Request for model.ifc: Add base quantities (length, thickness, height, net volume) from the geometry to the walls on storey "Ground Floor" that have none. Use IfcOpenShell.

First a look at what the model holds.

```python
import ifcopenshell
import ifcopenshell.util.element
import ifcopenshell.util.unit

model = ifcopenshell.open("model.ifc")
print(model.schema)
for unit_type in ("LENGTHUNIT", "AREAUNIT", "VOLUMEUNIT"):
    print(unit_type, ifcopenshell.util.unit.calculate_unit_scale(model, unit_type))
storey = next(s for s in model.by_type("IfcBuildingStorey") if s.Name == "Ground Floor")
walls = [e for e in ifcopenshell.util.element.get_decomposition(storey) if e.is_a("IfcWall")]
for e in sorted(walls, key=lambda e: e.id()):
    print(e.id(), e.is_a(), e.Name, list(ifcopenshell.util.element.get_psets(e, qtos_only=True)), sep=" | ")
```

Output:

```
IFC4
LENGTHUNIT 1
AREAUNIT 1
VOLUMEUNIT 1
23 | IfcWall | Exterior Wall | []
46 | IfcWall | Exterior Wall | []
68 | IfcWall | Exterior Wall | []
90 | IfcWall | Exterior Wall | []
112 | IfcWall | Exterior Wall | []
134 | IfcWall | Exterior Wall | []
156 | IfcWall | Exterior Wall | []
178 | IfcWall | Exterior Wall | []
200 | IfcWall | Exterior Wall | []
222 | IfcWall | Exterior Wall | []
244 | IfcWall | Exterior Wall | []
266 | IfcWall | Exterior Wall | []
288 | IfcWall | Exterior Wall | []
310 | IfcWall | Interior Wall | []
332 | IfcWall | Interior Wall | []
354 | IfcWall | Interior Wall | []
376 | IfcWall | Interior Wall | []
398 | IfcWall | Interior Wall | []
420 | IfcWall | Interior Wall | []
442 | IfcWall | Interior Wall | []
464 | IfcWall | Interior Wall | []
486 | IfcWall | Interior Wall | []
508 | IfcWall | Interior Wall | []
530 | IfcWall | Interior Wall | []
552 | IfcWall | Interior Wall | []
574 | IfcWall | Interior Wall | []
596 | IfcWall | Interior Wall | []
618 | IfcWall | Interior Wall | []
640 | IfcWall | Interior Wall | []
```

```python
import ifcopenshell
import ifcopenshell.api.pset
import ifcopenshell.geom
import ifcopenshell.util.element
import ifcopenshell.util.shape
import ifcopenshell.util.unit

model = ifcopenshell.open("model.ifc")
unit_scale = ifcopenshell.util.unit.calculate_unit_scale(model)
volume_scale = ifcopenshell.util.unit.calculate_unit_scale(model, "VOLUMEUNIT")
settings = ifcopenshell.geom.settings()

storey = next(s for s in model.by_type("IfcBuildingStorey") if s.Name == "Ground Floor")
walls = [e for e in ifcopenshell.util.element.get_decomposition(storey) if e.is_a("IfcWall")]

for e in sorted(walls, key=lambda e: e.id()):
    if ifcopenshell.util.element.get_psets(e, qtos_only=True, should_inherit=False):
        continue
    # Geometry comes back in metres, in the element's own axes.
    shape = ifcopenshell.geom.create_shape(settings, e)
    values = {
        "Length": ifcopenshell.util.shape.get_x(shape.geometry) / unit_scale,
        "Width": ifcopenshell.util.shape.get_y(shape.geometry) / unit_scale,
        "Height": ifcopenshell.util.shape.get_z(shape.geometry) / unit_scale,
        "NetVolume": ifcopenshell.util.shape.get_volume(shape.geometry) / volume_scale,
    }
    qto = ifcopenshell.api.pset.add_qto(model, product=e, name="Qto_WallBaseQuantities")
    ifcopenshell.api.pset.edit_qto(model, qto=qto, properties=values)
    print(e.id(), {k: round(v, 3) for k, v in values.items()})

model.write("model_rev.ifc")
```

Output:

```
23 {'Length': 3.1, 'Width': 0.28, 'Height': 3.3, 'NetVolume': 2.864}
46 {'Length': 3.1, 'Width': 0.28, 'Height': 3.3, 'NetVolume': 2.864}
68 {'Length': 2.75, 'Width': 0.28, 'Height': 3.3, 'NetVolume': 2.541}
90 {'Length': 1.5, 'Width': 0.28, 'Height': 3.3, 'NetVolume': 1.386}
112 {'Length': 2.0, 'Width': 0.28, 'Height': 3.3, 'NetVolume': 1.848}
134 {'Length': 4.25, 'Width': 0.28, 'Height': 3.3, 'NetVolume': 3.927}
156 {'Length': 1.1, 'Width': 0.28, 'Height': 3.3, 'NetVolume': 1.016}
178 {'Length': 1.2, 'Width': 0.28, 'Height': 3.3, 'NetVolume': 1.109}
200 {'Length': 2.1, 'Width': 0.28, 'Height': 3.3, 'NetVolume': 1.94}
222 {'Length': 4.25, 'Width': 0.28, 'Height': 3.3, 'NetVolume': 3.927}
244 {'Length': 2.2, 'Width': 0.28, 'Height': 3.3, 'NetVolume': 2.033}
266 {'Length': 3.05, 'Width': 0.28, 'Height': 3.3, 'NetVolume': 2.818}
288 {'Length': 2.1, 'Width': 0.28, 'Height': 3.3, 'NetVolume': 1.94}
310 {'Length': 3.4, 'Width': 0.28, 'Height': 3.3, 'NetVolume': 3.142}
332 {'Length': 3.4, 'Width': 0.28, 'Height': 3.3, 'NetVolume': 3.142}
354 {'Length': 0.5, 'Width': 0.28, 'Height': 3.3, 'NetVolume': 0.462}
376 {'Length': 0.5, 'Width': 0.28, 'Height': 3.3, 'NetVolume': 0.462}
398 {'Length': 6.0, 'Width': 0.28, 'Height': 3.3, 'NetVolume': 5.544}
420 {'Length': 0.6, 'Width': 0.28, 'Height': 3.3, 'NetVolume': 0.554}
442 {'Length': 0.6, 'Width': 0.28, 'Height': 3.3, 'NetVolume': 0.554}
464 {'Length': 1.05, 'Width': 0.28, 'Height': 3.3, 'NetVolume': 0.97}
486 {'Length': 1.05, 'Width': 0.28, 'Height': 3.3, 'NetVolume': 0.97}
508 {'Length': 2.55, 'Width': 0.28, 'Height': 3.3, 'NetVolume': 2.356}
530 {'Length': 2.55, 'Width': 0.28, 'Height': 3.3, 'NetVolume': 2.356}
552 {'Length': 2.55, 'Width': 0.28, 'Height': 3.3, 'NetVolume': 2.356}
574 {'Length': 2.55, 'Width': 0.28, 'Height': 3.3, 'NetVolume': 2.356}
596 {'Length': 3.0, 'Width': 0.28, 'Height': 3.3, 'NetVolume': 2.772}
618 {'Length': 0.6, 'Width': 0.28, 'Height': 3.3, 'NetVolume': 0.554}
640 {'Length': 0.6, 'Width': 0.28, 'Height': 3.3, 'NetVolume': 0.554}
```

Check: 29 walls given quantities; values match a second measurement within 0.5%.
